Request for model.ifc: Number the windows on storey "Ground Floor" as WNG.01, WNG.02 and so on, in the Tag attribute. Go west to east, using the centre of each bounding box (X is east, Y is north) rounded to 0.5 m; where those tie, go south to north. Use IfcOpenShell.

First a look at what the model holds.

```python
import ifcopenshell
import ifcopenshell.util.element
import ifcopenshell.util.placement

model = ifcopenshell.open("model.ifc")
print(model.schema)
storey = next(s for s in model.by_type("IfcBuildingStorey") if s.Name == "Ground Floor")
windows = [e for e in ifcopenshell.util.element.get_decomposition(storey) if e.is_a("IfcWindow")]
for e in sorted(windows, key=lambda e: e.id()):
    origin = ifcopenshell.util.placement.get_local_placement(e.ObjectPlacement)[:3, 3]
    print(e.id(), e.Tag, e.Name, origin.round(2) + 0.0, sep=" | ")
```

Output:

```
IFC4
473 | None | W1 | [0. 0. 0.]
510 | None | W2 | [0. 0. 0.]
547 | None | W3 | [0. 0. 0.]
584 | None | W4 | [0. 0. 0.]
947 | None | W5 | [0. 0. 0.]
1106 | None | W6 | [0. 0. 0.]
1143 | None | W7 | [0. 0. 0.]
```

```python
import ifcopenshell
import ifcopenshell.geom
import ifcopenshell.util.element
import ifcopenshell.util.shape

model = ifcopenshell.open("model.ifc")
settings = ifcopenshell.geom.settings()
settings.set("use-world-coords", True)


def centre(element):
    shape = ifcopenshell.geom.create_shape(settings, element)
    return ifcopenshell.util.shape.get_bbox_centroid(shape.geometry)


storey = next(s for s in model.by_type("IfcBuildingStorey") if s.Name == "Ground Floor")
windows = [e for e in ifcopenshell.util.element.get_decomposition(storey) if e.is_a("IfcWindow")]

# Insertion points can sit at a corner or the storey origin, so sort by the geometry (in metres).
centres = {e: centre(e) for e in windows}
windows.sort(key=lambda e: (round(centres[e][0] / 0.5), centres[e][1]))

for i, e in enumerate(windows, start=1):
    number = f"WNG.{i:02d}"
    e.Tag = number
    print(e.id(), number)

model.write("model-out.ifc")
```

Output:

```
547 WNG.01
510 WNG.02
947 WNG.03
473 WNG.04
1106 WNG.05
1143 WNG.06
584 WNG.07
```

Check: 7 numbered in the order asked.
